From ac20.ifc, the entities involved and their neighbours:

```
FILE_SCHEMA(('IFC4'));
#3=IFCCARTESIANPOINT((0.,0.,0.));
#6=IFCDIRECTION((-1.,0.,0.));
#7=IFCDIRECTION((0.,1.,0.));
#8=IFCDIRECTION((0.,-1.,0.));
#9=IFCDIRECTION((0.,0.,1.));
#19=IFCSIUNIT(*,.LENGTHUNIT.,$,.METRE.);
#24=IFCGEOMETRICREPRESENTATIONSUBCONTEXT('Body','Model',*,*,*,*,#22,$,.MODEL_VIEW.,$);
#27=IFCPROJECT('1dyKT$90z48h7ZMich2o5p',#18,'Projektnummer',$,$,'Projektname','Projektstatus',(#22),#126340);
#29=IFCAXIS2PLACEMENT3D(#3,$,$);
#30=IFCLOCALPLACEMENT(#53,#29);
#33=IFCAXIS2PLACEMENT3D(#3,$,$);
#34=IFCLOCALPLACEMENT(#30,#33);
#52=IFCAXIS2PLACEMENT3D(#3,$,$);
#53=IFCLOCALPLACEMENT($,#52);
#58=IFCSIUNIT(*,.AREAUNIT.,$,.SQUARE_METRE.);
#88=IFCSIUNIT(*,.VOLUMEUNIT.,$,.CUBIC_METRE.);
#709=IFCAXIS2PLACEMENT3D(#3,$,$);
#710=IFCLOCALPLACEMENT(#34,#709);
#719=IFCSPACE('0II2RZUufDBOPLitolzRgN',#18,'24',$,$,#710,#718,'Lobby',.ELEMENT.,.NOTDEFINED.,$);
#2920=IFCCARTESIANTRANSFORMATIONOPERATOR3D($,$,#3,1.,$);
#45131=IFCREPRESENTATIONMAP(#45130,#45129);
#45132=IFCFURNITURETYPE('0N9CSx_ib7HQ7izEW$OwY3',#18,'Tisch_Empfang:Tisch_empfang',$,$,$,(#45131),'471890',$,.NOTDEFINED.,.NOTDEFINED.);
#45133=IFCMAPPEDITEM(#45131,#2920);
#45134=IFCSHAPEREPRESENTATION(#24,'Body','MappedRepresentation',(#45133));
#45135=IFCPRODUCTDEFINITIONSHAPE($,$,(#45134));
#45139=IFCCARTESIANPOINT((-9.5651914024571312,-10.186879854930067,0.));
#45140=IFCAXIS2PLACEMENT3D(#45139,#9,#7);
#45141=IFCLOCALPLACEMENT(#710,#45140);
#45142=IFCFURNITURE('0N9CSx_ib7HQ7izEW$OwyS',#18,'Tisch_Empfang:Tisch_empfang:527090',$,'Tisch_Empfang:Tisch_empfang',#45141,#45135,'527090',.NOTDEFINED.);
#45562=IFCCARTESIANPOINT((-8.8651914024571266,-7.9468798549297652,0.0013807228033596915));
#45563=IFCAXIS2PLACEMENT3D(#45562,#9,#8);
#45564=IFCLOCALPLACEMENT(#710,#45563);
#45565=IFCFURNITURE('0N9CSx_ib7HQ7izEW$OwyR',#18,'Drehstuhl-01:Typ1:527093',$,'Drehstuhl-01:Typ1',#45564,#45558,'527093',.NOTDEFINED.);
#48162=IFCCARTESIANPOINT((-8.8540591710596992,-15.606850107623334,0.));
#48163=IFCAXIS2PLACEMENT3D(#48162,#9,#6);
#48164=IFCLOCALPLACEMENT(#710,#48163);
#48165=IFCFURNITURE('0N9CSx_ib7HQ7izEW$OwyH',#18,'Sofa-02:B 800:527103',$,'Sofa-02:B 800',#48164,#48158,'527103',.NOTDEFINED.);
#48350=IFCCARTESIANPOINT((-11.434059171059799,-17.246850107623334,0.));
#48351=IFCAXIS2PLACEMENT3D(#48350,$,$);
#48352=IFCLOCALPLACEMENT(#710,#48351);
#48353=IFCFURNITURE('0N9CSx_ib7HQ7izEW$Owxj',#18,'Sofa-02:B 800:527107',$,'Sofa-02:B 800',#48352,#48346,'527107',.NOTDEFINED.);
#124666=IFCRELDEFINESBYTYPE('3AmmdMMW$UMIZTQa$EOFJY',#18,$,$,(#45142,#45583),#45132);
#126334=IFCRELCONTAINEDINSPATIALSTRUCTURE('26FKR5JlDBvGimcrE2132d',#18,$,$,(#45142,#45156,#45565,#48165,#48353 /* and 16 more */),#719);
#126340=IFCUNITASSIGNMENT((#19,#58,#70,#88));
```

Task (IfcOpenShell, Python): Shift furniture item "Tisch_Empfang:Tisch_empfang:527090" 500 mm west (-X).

```python
import ifcopenshell
import ifcopenshell.api.geometry
import ifcopenshell.util.placement

model = ifcopenshell.open("ac20.ifc")

item = model.by_id(45142)
matrix = ifcopenshell.util.placement.get_local_placement(item.ObjectPlacement)
matrix[0, 3] -= 0.5
ifcopenshell.api.geometry.edit_object_placement(model, product=item, matrix=matrix, is_si=False)

print(ifcopenshell.util.placement.get_local_placement(item.ObjectPlacement).round(3) + 0.0)

model.write("ac20_updated.ifc")
```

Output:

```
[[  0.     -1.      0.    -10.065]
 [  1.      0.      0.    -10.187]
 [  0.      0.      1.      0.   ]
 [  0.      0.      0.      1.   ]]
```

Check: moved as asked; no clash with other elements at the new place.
